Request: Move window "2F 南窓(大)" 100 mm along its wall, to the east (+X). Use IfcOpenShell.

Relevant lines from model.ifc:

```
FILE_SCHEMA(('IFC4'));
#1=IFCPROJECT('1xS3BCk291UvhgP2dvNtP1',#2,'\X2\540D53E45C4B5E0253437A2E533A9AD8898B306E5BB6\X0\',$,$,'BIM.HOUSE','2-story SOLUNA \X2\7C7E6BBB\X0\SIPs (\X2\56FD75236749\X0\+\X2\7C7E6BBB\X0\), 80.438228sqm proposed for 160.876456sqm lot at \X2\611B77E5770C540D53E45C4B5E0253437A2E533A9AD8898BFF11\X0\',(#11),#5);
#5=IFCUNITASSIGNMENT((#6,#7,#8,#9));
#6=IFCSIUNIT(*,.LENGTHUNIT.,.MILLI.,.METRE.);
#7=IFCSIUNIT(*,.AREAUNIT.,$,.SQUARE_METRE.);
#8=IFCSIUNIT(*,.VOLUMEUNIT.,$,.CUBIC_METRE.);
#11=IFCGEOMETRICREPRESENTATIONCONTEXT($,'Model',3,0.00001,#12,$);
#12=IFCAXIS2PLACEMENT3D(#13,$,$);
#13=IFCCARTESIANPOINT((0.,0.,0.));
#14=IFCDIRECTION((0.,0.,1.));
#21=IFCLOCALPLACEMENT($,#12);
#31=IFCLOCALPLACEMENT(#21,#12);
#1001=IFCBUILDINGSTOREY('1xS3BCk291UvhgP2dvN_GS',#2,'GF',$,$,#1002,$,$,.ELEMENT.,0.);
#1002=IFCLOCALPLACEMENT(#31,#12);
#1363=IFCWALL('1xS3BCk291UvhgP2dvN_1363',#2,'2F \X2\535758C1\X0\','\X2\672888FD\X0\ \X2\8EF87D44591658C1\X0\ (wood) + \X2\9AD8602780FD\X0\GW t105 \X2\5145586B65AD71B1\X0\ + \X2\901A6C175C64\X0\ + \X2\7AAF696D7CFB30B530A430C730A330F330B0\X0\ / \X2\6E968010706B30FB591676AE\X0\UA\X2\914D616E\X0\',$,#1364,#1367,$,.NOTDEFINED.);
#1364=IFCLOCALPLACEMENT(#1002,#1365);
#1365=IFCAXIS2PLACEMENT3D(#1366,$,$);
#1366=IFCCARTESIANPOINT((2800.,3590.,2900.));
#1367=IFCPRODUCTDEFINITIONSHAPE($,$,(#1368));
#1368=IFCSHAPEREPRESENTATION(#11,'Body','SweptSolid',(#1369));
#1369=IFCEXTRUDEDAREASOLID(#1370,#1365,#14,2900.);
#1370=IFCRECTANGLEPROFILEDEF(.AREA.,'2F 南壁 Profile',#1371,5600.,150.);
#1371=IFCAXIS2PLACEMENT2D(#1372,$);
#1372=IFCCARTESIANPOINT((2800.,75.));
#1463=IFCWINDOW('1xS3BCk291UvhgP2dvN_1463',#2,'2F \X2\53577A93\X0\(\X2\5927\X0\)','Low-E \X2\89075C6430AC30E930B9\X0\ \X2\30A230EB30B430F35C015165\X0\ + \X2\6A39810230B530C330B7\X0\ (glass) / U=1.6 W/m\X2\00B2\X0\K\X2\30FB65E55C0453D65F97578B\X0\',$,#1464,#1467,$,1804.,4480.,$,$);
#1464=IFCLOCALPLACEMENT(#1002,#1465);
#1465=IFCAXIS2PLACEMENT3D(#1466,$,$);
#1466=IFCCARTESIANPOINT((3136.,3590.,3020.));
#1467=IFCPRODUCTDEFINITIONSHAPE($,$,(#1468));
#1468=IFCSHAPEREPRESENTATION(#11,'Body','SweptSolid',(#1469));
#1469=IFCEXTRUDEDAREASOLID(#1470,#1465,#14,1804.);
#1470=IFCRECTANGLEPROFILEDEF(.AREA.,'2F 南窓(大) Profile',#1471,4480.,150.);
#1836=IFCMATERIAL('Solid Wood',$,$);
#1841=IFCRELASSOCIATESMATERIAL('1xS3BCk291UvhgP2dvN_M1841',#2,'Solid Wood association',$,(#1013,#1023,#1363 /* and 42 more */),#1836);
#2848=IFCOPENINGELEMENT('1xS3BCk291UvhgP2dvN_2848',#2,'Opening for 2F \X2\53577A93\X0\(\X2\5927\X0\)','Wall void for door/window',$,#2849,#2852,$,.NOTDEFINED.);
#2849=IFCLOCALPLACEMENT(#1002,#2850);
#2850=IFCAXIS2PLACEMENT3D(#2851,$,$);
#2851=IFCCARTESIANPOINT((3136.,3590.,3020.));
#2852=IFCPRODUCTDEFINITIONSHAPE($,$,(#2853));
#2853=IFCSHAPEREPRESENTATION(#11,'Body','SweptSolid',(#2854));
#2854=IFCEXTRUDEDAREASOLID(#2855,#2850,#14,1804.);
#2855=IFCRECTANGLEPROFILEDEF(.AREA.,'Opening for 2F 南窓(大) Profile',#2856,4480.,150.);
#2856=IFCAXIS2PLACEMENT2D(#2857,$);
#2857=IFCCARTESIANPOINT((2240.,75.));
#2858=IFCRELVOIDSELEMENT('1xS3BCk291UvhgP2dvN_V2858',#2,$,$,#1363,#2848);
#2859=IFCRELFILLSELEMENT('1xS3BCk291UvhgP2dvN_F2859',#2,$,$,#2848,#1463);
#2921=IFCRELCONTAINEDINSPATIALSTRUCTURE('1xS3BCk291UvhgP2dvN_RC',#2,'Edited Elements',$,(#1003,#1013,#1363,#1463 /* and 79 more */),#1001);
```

```python
import ifcopenshell
import ifcopenshell.api.geometry
import ifcopenshell.util.placement
import ifcopenshell.util.unit

model = ifcopenshell.open("model.ifc")
unit_scale = ifcopenshell.util.unit.calculate_unit_scale(model)

window = model.by_guid("1xS3BCk291UvhgP2dvN_1463")
opening = window.FillsVoids[0].RelatingOpeningElement
wall = opening.VoidsElements[0].RelatingBuildingElement

wall_matrix = ifcopenshell.util.placement.get_local_placement(wall.ObjectPlacement)
shift = wall_matrix[:3, 0] * 0.1 / unit_scale
before = ifcopenshell.util.placement.get_local_placement(window.ObjectPlacement)[:3, 3].copy()

# The window is not placed relative to its opening, so move both.
for product in (opening, window):
    matrix = ifcopenshell.util.placement.get_local_placement(product.ObjectPlacement)
    matrix[:3, 3] += shift
    ifcopenshell.api.geometry.edit_object_placement(model, product=product, matrix=matrix, is_si=False)

after = ifcopenshell.util.placement.get_local_placement(window.ObjectPlacement)[:3, 3]
print("window moved by", (after - before).round(3) + 0.0)

model.write("model_edited.ifc")
```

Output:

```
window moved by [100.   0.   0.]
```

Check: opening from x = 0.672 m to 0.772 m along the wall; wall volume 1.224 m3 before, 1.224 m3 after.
